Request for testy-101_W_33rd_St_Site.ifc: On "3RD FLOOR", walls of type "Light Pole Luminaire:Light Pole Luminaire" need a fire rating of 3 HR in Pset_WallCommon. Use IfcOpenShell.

First a look at what the model holds.

```python
import ifcopenshell
import ifcopenshell.util.element

model = ifcopenshell.open("testy-101_W_33rd_St_Site.ifc")
print(model.schema)
storey = next(s for s in model.by_type("IfcBuildingStorey") if s.Name == "3RD FLOOR")
walls = [e for e in ifcopenshell.util.element.get_decomposition(storey) if e.is_a("IfcWall")]
seen = {}
for e in walls:
    element_type = ifcopenshell.util.element.get_type(e)
    key = (element_type.Name if element_type != e and element_type else None, ifcopenshell.util.element.get_pset(e, "Pset_WallCommon", "FireRating"))
    seen[key] = seen.get(key, 0) + 1
for (name, value), count in sorted(seen.items(), key=str):
    print(count, "x", name, "|", value)
```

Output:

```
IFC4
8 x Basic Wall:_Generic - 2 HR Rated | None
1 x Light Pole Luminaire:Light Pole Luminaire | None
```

```python
import ifcopenshell
import ifcopenshell.api.pset
import ifcopenshell.util.element

model = ifcopenshell.open("testy-101_W_33rd_St_Site.ifc")

storey = next(s for s in model.by_type("IfcBuildingStorey") if s.Name == "3RD FLOOR")
walls = [e for e in ifcopenshell.util.element.get_decomposition(storey) if e.is_a("IfcWall")]

count = 0
for e in walls:
    element_type = ifcopenshell.util.element.get_type(e)
    if element_type in (None, e) or element_type.Name != "Light Pole Luminaire:Light Pole Luminaire":
        continue
    # add_pset returns the element's existing set when there is one.
    pset = ifcopenshell.api.pset.add_pset(model, product=e, name="Pset_WallCommon")
    ifcopenshell.api.pset.edit_pset(model, pset=pset, properties={"FireRating": "3 HR"})
    count += 1

print(count, "walls updated")

model.write("testy-101_W_33rd_St_Site_rev.ifc")
```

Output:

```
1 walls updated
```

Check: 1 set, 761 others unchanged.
